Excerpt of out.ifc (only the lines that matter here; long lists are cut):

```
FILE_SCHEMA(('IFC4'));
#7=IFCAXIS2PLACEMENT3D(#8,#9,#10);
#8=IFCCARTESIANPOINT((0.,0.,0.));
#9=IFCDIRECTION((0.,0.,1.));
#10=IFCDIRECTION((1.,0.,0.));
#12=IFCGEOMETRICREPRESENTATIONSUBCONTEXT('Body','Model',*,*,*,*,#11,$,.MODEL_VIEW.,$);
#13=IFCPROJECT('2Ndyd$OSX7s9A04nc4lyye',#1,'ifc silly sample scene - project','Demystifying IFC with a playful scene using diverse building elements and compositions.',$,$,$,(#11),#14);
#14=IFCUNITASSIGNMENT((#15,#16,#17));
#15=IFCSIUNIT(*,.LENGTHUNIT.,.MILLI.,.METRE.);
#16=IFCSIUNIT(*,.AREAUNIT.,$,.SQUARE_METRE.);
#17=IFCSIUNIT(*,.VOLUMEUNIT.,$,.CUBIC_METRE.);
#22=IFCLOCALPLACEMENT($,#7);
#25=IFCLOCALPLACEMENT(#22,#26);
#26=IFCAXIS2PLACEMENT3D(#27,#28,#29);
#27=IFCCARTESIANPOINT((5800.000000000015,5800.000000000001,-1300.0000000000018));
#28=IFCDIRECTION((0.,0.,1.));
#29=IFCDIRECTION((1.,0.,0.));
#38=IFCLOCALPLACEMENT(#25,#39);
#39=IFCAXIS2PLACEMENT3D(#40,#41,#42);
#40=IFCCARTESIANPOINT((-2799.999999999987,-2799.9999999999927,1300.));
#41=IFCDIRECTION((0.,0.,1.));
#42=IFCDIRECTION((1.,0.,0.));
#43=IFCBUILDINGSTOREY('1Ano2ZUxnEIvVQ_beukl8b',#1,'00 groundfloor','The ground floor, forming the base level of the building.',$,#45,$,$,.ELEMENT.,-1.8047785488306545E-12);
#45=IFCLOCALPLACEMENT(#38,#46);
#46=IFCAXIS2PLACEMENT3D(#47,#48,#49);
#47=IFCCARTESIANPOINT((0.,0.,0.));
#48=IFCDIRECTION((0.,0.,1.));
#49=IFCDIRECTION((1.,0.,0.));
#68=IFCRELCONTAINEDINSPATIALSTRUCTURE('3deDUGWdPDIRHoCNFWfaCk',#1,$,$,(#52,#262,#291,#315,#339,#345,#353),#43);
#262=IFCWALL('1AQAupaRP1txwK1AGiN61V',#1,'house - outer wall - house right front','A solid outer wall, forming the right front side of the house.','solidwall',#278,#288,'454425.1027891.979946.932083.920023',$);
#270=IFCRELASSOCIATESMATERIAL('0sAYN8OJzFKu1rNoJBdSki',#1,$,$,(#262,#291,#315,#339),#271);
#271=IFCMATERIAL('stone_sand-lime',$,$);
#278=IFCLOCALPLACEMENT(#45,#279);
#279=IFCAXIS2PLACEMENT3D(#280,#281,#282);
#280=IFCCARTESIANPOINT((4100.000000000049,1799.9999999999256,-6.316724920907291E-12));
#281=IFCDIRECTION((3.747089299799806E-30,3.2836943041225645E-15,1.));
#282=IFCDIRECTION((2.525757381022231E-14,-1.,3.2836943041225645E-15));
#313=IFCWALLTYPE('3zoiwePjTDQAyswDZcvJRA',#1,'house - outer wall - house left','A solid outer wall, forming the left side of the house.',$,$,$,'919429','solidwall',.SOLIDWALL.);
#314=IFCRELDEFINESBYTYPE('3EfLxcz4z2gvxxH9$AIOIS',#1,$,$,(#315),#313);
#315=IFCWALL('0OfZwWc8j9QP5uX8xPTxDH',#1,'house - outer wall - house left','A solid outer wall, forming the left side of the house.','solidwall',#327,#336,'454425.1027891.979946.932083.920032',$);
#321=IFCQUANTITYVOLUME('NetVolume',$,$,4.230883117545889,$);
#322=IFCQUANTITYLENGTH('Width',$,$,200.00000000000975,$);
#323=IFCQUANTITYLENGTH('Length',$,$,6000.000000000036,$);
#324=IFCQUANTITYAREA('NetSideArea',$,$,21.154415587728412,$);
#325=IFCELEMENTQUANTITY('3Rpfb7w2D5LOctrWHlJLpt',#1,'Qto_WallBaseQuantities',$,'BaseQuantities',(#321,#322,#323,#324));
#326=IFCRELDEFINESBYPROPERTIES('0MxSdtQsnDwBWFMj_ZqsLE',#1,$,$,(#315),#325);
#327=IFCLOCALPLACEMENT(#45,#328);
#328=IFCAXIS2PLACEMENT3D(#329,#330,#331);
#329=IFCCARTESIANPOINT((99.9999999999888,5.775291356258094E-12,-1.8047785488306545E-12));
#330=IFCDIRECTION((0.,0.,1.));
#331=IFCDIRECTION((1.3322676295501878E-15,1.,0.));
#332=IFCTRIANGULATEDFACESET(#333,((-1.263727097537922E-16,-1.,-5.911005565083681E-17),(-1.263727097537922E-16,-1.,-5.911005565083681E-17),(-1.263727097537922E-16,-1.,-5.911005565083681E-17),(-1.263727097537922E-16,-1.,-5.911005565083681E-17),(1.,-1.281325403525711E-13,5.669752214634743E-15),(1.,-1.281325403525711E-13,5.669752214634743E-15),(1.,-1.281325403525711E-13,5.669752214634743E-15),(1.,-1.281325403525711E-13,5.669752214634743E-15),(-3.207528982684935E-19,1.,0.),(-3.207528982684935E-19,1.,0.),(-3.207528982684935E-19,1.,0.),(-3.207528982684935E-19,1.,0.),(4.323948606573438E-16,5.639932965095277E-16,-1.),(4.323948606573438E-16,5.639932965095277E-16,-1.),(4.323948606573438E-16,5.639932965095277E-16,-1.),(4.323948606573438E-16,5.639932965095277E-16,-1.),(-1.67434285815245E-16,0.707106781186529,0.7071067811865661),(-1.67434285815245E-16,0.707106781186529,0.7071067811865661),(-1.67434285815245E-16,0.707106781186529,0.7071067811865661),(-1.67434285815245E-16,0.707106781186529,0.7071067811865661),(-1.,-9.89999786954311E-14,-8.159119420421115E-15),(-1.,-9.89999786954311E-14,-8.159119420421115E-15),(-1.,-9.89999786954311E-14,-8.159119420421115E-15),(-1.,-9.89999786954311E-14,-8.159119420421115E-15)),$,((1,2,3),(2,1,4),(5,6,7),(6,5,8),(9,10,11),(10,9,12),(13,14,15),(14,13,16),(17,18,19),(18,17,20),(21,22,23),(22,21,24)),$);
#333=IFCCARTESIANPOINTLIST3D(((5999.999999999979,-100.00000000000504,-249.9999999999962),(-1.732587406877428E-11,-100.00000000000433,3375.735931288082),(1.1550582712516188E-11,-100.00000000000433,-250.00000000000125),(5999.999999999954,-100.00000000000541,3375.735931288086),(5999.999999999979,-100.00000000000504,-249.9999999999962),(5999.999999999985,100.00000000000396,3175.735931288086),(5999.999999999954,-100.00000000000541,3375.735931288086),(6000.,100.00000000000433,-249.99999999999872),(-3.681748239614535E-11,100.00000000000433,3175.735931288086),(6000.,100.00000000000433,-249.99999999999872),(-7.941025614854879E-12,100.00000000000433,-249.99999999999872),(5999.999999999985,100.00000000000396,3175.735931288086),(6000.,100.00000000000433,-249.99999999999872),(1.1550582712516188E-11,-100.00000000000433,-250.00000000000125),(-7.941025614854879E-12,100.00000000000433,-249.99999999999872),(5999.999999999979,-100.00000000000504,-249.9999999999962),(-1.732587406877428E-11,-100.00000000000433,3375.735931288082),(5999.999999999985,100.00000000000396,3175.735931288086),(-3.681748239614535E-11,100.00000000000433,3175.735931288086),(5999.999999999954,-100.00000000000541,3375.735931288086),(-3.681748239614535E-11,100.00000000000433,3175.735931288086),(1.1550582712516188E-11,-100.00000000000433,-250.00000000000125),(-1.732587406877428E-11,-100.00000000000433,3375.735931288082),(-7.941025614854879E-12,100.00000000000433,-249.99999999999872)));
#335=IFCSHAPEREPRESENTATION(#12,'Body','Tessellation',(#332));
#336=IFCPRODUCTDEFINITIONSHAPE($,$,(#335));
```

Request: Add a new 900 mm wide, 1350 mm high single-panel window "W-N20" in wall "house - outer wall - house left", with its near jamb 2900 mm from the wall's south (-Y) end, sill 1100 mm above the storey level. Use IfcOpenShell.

```python
import numpy as np
import ifcopenshell
import ifcopenshell.api.feature
import ifcopenshell.api.geometry
import ifcopenshell.api.pset
import ifcopenshell.api.root
import ifcopenshell.api.spatial
import ifcopenshell.geom
import ifcopenshell.util.element
import ifcopenshell.util.placement
import ifcopenshell.util.representation
import ifcopenshell.util.shape
import ifcopenshell.util.unit

model = ifcopenshell.open("out.ifc")
unit_scale = ifcopenshell.util.unit.calculate_unit_scale(model)
area_scale = ifcopenshell.util.unit.calculate_unit_scale(model, "AREAUNIT")
volume_scale = ifcopenshell.util.unit.calculate_unit_scale(model, "VOLUMEUNIT")
settings = ifcopenshell.geom.settings()


def volume(element):
    """Net volume in cubic metres, openings subtracted."""
    shape = ifcopenshell.geom.create_shape(settings, element)
    return ifcopenshell.util.shape.get_volume(shape.geometry)


wall = model.by_guid("0OfZwWc8j9QP5uX8xPTxDH")
storey = ifcopenshell.util.element.get_container(wall, ifc_class="IfcBuildingStorey")
context = ifcopenshell.util.representation.get_context(model, "Model", "Body", "MODEL_VIEW")
before = volume(wall)

width, height, from_end, sill = 0.9, 1.35, 2.9, 1.1  # metres

# The wall runs along its own X axis, and the end named is its -X end.
wall_shape = ifcopenshell.geom.create_shape(settings, wall)
x, y, z = ifcopenshell.util.shape.get_vertices(wall_shape.geometry).T
start = x.min() + from_end
face, thickness = float(y.min()), float(y.max() - y.min())
wall_matrix = ifcopenshell.util.placement.get_local_placement(wall.ObjectPlacement)
level = ifcopenshell.util.placement.get_local_placement(storey.ObjectPlacement)[2, 3]


def in_wall(x, y):
    """Placement at x, y metres in the wall's axes, at sill height."""
    matrix = wall_matrix.copy()
    matrix[:, 3] = wall_matrix @ np.array([x / unit_scale, y / unit_scale, 0.0, 1.0])
    matrix[2, 3] = level + sill / unit_scale
    return matrix


# Opening: a box that overshoots both wall faces by 50 mm.
opening = ifcopenshell.api.root.create_entity(model, ifc_class="IfcOpeningElement", predefined_type="OPENING")
box = ifcopenshell.api.geometry.add_wall_representation(
    model, context=context, length=width, height=height, thickness=thickness + 0.1
)
ifcopenshell.api.geometry.assign_representation(model, product=opening, representation=box)
ifcopenshell.api.geometry.edit_object_placement(model, product=opening, matrix=in_wall(start, face - 0.05), is_si=False)
ifcopenshell.api.feature.add_feature(model, feature=opening, element=wall)

window = ifcopenshell.api.root.create_entity(model, ifc_class="IfcWindow", name="W-N20", predefined_type="WINDOW")
window.OverallWidth, window.OverallHeight = width / unit_scale, height / unit_scale
window.PartitioningType = "SINGLE_PANEL"
body = ifcopenshell.api.geometry.add_window_representation(
    model,
    context=context,
    overall_width=window.OverallWidth,
    overall_height=window.OverallHeight,
    partition_type="SINGLE_PANEL",
)
ifcopenshell.api.geometry.assign_representation(model, product=window, representation=body)
ifcopenshell.api.spatial.assign_container(model, products=[window], relating_structure=storey)
ifcopenshell.api.feature.add_filling(model, opening=opening, element=window)

# Centre the window in the wall's thickness.
ifcopenshell.api.geometry.edit_object_placement(model, product=window, matrix=in_wall(start, face), is_si=False)
window_shape = ifcopenshell.geom.create_shape(settings, window)
depth = ifcopenshell.util.shape.get_vertices(window_shape.geometry)[:, 1]
offset = face + thickness / 2 - (depth.min() + depth.max()) / 2
ifcopenshell.api.geometry.edit_object_placement(model, product=window, matrix=in_wall(start, offset), is_si=False)

after = volume(wall)

# Update the wall's stored quantities.
qto = model.by_id(ifcopenshell.util.element.get_pset(wall, "Qto_WallBaseQuantities", should_inherit=False)["id"])
ifcopenshell.api.pset.edit_qto(model, qto=qto, properties={
    "NetVolume": after / volume_scale,
    "NetSideArea": after / thickness / area_scale,
})

print(f"wall volume {before:.3f} -> {after:.3f} m3")

model.write("out_rev.ifc")
```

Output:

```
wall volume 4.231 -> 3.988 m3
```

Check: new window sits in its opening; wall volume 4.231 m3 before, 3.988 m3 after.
